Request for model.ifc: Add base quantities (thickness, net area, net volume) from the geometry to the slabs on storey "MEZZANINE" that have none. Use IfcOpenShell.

First a look at what the model holds.

```python
import ifcopenshell
import ifcopenshell.util.element
import ifcopenshell.util.unit

model = ifcopenshell.open("model.ifc")
print(model.schema)
for unit_type in ("LENGTHUNIT", "AREAUNIT", "VOLUMEUNIT"):
    print(unit_type, ifcopenshell.util.unit.calculate_unit_scale(model, unit_type))
storey = next(s for s in model.by_type("IfcBuildingStorey") if s.Name == "MEZZANINE")
slabs = [e for e in ifcopenshell.util.element.get_decomposition(storey) if e.is_a("IfcSlab")]
for e in sorted(slabs, key=lambda e: e.id()):
    print(e.id(), e.is_a(), e.Name, list(ifcopenshell.util.element.get_psets(e, qtos_only=True)), sep=" | ")
```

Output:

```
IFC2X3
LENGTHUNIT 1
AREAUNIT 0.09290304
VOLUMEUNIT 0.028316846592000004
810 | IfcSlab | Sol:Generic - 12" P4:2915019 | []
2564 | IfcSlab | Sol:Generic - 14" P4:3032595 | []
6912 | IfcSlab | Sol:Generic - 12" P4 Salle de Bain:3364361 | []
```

```python
import ifcopenshell
import ifcopenshell.api.pset
import ifcopenshell.geom
import ifcopenshell.util.element
import ifcopenshell.util.shape
import ifcopenshell.util.unit

model = ifcopenshell.open("model.ifc")
unit_scale = ifcopenshell.util.unit.calculate_unit_scale(model)
area_scale = ifcopenshell.util.unit.calculate_unit_scale(model, "AREAUNIT")
volume_scale = ifcopenshell.util.unit.calculate_unit_scale(model, "VOLUMEUNIT")
settings = ifcopenshell.geom.settings()

storey = next(s for s in model.by_type("IfcBuildingStorey") if s.Name == "MEZZANINE")
slabs = [e for e in ifcopenshell.util.element.get_decomposition(storey) if e.is_a("IfcSlab")]

for e in sorted(slabs, key=lambda e: e.id()):
    if ifcopenshell.util.element.get_psets(e, qtos_only=True, should_inherit=False):
        continue
    # Geometry comes back in metres, in the element's own axes.
    shape = ifcopenshell.geom.create_shape(settings, e)
    values = {
        "Width": ifcopenshell.util.shape.get_z(shape.geometry) / unit_scale,
        "NetArea": ifcopenshell.util.shape.get_footprint_area(shape.geometry) / area_scale,
        "NetVolume": ifcopenshell.util.shape.get_volume(shape.geometry) / volume_scale,
    }
    qto = ifcopenshell.api.pset.add_qto(model, product=e, name="BaseQuantities")
    ifcopenshell.api.pset.edit_qto(model, qto=qto, properties=values)
    print(e.id(), {k: round(v, 3) for k, v in values.items()})

model.write("model-out.ifc")
```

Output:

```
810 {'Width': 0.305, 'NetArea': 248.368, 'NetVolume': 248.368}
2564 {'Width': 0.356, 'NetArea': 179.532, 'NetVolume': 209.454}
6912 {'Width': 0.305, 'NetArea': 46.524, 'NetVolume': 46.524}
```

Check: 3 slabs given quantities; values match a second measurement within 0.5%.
